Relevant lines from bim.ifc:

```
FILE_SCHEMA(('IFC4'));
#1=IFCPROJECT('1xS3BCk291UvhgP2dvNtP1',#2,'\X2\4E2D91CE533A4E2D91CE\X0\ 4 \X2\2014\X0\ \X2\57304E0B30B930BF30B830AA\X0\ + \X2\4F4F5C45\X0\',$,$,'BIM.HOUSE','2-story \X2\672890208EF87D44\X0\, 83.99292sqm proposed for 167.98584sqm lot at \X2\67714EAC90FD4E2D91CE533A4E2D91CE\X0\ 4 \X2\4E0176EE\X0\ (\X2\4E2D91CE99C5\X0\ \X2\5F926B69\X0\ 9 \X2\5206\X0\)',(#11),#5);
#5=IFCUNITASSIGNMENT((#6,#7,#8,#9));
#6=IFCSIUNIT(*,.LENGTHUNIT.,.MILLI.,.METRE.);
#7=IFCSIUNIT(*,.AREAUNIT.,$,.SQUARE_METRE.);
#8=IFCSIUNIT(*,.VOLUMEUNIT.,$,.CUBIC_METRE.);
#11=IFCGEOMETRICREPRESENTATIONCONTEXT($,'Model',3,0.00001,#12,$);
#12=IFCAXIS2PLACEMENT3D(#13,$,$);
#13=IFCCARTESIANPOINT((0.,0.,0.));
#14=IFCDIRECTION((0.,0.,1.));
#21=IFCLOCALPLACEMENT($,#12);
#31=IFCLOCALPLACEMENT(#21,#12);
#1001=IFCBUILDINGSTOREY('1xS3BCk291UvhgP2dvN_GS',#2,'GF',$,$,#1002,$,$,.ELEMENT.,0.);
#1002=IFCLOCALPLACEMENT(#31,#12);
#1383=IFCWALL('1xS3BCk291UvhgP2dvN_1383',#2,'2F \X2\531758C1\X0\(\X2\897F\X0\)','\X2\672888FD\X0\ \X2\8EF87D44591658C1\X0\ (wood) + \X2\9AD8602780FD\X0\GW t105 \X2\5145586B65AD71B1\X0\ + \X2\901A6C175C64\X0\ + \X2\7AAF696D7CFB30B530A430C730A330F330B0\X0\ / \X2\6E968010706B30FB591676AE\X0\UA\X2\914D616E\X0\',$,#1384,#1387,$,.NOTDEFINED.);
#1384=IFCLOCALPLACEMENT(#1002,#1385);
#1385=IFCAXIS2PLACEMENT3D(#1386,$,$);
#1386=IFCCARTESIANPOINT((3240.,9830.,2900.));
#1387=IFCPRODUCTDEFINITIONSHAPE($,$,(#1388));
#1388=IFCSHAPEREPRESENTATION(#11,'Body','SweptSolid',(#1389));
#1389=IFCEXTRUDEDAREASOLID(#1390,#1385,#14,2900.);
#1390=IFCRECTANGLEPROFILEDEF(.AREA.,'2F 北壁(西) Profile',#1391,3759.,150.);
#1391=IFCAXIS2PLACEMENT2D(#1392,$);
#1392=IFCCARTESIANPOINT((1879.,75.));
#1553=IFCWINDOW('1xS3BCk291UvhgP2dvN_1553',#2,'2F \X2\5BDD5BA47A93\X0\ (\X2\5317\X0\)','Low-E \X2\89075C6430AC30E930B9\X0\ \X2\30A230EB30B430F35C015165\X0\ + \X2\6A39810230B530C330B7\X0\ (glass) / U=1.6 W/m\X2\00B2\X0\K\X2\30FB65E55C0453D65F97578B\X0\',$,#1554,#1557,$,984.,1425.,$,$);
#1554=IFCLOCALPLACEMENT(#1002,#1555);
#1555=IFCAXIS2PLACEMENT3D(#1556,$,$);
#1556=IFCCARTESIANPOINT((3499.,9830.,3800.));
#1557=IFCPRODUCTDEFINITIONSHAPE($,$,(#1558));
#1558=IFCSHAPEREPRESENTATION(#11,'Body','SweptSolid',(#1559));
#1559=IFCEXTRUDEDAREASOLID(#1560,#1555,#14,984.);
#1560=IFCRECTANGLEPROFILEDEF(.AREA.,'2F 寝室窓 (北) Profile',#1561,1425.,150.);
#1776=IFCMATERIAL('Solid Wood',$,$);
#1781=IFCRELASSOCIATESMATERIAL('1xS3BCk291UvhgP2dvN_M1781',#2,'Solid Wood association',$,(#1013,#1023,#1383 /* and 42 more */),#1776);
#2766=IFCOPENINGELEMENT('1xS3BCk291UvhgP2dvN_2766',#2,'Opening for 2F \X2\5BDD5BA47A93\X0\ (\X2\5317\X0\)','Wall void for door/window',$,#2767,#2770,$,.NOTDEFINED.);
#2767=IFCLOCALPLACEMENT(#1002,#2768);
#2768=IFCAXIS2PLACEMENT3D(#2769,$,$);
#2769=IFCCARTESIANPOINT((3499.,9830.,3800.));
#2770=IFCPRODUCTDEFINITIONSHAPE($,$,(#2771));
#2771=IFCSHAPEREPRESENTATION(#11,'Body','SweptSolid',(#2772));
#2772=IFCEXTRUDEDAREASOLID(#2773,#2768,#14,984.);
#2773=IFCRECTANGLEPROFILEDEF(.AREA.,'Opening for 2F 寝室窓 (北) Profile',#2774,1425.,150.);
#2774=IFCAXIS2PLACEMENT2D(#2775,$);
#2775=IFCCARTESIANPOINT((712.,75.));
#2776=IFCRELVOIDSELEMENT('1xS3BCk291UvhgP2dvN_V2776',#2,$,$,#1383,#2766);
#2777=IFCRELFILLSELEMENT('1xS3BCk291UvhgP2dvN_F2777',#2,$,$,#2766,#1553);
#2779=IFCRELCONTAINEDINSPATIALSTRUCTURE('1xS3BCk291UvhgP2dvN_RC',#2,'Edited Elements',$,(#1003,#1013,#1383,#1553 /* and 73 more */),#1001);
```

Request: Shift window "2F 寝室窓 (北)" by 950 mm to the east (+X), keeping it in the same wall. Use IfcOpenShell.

```python
import ifcopenshell
import ifcopenshell.api.geometry
import ifcopenshell.util.placement
import ifcopenshell.util.unit

model = ifcopenshell.open("bim.ifc")
unit_scale = ifcopenshell.util.unit.calculate_unit_scale(model)

window = model.by_id(1553)
opening = window.FillsVoids[0].RelatingOpeningElement
wall = opening.VoidsElements[0].RelatingBuildingElement

wall_matrix = ifcopenshell.util.placement.get_local_placement(wall.ObjectPlacement)
shift = wall_matrix[:3, 0] * 0.95 / unit_scale
before = ifcopenshell.util.placement.get_local_placement(window.ObjectPlacement)[:3, 3].copy()

# The window is not placed relative to its opening, so move both.
for product in (opening, window):
    matrix = ifcopenshell.util.placement.get_local_placement(product.ObjectPlacement)
    matrix[:3, 3] += shift
    ifcopenshell.api.geometry.edit_object_placement(model, product=product, matrix=matrix, is_si=False)

after = ifcopenshell.util.placement.get_local_placement(window.ObjectPlacement)[:3, 3]
print("window moved by", (after - before).round(3) + 0.0)

model.write("bim_rev.ifc")
```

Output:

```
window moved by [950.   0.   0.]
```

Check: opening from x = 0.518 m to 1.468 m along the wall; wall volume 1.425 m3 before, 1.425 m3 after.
